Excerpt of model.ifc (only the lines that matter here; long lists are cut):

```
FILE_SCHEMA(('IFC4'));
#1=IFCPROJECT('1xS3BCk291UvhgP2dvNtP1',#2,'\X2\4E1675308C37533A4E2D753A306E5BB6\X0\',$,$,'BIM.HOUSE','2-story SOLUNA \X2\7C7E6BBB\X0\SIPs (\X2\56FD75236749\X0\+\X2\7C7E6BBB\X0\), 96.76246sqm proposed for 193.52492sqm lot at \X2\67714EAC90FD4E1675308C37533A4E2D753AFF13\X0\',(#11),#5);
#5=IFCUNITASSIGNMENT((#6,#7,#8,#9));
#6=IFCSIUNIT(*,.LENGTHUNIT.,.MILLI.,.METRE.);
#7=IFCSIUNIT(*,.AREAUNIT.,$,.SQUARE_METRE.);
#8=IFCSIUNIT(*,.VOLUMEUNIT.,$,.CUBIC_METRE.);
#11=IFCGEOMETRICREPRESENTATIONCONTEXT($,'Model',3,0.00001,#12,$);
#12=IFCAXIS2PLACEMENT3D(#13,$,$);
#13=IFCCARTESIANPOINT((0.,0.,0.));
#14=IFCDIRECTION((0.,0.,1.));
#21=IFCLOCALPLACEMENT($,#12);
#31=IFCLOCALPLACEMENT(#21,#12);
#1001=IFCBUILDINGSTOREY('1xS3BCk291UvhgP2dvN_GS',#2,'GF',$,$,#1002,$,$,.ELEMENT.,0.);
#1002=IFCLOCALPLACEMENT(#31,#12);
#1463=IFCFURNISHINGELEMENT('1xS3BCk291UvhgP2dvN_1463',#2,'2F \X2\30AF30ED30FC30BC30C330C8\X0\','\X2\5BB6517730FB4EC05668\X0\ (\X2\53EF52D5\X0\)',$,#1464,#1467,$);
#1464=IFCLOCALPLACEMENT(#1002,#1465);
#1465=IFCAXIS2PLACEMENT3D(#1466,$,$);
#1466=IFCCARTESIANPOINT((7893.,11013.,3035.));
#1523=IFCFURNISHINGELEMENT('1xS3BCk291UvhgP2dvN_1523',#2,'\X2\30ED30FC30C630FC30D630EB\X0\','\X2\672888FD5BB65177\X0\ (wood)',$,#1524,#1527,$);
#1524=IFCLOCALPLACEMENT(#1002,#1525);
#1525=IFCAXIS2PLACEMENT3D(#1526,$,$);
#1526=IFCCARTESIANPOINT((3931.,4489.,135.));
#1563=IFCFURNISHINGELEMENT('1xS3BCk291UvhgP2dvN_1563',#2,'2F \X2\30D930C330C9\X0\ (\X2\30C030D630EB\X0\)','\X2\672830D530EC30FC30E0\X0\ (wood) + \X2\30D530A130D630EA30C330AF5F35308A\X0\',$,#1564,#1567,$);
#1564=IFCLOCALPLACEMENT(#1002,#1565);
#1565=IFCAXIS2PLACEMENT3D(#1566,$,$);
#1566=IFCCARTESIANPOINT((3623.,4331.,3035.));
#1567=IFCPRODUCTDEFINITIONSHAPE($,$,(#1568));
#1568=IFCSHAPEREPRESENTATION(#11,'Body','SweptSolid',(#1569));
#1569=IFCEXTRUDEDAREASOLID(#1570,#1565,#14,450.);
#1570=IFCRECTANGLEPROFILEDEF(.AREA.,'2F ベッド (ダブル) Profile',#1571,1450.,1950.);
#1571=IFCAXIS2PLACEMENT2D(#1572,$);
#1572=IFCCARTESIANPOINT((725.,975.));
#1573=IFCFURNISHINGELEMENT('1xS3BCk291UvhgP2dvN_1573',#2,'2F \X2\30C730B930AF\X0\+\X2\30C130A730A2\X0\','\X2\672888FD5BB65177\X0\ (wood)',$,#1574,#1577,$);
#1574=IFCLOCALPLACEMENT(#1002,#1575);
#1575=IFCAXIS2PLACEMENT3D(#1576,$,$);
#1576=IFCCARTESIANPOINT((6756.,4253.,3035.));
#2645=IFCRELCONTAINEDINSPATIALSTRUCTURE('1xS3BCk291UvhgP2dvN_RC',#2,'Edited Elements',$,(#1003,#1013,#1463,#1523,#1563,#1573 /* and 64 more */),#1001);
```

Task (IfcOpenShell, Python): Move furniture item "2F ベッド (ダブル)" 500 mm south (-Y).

```python
import ifcopenshell
import ifcopenshell.api.geometry
import ifcopenshell.util.placement

model = ifcopenshell.open("model.ifc")

item = model.by_guid("1xS3BCk291UvhgP2dvN_1563")
matrix = ifcopenshell.util.placement.get_local_placement(item.ObjectPlacement)
matrix[1, 3] -= 500.0
ifcopenshell.api.geometry.edit_object_placement(model, product=item, matrix=matrix, is_si=False)

print(ifcopenshell.util.placement.get_local_placement(item.ObjectPlacement).round(3) + 0.0)

model.write("model_v2.ifc")
```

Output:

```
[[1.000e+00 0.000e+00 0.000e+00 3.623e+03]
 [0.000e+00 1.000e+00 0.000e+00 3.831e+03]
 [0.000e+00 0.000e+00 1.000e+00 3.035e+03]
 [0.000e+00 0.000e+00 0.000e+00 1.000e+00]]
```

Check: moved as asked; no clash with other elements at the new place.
